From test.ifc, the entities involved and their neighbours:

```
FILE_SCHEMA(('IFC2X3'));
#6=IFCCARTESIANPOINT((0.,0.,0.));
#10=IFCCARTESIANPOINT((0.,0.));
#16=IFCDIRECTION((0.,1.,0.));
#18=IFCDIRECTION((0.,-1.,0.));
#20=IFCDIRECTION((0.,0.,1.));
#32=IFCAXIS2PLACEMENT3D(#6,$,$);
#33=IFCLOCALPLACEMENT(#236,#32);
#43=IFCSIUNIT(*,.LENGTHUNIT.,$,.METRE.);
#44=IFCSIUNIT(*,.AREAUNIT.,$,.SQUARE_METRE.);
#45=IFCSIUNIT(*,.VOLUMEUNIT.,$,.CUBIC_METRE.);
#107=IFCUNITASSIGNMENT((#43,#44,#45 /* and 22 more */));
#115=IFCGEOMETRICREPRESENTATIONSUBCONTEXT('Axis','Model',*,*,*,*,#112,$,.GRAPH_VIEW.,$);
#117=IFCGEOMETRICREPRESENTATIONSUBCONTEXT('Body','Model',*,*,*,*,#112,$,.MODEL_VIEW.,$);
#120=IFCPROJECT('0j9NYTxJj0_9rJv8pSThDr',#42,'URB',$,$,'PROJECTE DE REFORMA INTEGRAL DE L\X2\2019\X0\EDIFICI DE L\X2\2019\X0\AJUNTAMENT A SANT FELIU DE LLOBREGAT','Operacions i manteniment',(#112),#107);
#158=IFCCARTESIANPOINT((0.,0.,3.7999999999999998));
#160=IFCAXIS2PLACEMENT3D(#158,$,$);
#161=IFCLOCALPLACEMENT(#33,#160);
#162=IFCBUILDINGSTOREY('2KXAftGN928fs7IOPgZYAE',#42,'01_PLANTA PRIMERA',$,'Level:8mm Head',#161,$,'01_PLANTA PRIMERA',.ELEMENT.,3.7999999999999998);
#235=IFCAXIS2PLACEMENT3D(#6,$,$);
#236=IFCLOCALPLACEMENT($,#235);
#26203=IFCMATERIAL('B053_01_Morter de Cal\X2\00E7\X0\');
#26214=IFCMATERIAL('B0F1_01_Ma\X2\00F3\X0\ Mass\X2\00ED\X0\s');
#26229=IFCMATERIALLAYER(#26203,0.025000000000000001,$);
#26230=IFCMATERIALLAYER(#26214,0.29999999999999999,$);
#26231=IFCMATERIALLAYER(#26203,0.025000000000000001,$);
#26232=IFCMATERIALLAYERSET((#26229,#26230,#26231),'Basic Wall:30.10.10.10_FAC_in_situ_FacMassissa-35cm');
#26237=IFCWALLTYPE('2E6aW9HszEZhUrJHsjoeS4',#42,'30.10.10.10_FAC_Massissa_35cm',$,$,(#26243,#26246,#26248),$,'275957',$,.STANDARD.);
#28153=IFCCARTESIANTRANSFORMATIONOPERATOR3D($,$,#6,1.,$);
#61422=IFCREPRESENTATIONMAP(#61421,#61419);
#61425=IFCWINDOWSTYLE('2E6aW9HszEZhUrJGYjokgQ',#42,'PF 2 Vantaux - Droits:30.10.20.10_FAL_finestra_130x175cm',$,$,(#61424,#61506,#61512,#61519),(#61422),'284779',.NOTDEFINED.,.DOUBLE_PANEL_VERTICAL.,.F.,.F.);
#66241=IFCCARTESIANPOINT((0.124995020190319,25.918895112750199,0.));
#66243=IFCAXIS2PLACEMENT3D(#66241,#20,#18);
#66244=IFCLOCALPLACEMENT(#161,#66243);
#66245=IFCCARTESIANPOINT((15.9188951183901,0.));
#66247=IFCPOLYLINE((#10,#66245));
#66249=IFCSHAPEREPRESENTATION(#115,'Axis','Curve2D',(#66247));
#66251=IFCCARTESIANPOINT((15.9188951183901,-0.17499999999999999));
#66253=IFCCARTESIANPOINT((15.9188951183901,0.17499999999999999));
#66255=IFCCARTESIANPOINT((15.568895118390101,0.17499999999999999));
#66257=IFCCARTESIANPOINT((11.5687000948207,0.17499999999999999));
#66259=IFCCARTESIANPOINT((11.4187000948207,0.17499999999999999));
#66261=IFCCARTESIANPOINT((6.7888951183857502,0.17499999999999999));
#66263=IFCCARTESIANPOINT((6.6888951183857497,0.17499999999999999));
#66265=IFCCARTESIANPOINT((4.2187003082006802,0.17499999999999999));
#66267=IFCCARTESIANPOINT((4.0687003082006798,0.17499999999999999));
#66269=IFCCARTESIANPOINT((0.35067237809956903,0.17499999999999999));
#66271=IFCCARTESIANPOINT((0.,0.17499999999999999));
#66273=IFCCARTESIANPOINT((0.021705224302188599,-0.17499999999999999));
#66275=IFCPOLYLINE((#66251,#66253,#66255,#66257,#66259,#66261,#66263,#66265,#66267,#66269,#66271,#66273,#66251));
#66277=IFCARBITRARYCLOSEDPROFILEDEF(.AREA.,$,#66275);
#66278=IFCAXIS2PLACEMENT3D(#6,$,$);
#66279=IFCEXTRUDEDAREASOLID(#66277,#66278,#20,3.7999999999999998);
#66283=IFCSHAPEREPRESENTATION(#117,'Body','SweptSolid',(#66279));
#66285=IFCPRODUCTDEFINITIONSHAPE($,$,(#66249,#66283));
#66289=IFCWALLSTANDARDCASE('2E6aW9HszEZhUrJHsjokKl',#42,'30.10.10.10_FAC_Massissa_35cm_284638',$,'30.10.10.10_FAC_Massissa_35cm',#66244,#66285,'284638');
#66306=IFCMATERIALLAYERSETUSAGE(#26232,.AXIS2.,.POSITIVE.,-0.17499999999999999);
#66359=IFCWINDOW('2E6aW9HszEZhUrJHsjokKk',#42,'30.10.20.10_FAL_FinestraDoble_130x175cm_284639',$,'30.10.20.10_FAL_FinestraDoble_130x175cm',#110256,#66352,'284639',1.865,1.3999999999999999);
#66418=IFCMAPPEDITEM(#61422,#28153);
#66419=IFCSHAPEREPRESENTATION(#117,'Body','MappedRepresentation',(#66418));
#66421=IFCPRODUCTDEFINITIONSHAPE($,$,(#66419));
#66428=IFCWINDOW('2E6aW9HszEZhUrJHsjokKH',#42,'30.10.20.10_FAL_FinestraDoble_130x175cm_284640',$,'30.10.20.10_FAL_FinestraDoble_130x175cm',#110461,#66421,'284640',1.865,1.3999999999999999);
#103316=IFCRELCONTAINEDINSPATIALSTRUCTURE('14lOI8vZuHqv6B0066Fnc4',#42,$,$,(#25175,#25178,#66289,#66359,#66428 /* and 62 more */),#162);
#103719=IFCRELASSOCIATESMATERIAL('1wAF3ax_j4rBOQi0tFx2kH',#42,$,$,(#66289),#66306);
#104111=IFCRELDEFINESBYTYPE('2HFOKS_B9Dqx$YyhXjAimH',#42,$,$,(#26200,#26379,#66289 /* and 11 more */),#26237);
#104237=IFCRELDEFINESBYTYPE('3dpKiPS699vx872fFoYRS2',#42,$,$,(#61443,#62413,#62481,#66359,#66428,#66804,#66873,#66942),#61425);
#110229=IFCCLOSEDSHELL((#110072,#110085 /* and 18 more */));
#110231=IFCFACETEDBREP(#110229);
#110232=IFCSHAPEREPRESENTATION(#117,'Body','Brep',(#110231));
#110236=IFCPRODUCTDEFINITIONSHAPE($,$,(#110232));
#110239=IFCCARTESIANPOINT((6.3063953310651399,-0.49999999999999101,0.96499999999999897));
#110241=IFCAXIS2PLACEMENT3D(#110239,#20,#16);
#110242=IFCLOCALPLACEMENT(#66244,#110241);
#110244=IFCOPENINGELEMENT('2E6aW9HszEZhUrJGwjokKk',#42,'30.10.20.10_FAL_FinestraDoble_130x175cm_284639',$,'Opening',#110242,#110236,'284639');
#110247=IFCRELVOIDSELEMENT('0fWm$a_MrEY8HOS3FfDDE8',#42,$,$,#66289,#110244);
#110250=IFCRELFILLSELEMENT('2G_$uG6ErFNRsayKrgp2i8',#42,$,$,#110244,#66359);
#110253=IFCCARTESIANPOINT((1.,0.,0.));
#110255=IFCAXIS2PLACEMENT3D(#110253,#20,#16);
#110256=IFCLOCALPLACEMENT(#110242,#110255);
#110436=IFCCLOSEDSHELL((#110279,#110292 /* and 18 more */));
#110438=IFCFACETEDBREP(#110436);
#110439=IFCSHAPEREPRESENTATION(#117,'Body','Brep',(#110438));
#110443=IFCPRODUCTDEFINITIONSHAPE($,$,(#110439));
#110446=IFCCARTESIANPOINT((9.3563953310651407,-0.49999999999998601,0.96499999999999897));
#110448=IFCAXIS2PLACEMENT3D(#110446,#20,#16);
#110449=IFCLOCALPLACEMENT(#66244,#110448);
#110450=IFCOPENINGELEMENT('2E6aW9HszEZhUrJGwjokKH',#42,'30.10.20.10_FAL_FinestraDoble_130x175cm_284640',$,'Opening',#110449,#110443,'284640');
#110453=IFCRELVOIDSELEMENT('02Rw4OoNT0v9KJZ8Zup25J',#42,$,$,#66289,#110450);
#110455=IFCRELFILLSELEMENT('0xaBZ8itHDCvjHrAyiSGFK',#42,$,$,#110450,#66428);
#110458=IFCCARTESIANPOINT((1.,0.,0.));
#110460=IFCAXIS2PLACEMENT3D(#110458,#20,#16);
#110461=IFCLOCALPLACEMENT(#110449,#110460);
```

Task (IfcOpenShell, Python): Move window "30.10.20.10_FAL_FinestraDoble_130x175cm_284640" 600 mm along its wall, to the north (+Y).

```python
import ifcopenshell
import ifcopenshell.api.geometry
import ifcopenshell.util.placement
import ifcopenshell.util.unit

model = ifcopenshell.open("test.ifc")
unit_scale = ifcopenshell.util.unit.calculate_unit_scale(model)

window = model.by_guid("2E6aW9HszEZhUrJHsjokKH")
opening = window.FillsVoids[0].RelatingOpeningElement
wall = opening.VoidsElements[0].RelatingBuildingElement

wall_matrix = ifcopenshell.util.placement.get_local_placement(wall.ObjectPlacement)
shift = wall_matrix[:3, 0] * -0.6 / unit_scale
before = ifcopenshell.util.placement.get_local_placement(window.ObjectPlacement)[:3, 3].copy()

# The window is placed relative to its opening, so it follows when the opening moves.
matrix = ifcopenshell.util.placement.get_local_placement(opening.ObjectPlacement)
matrix[:3, 3] += shift
ifcopenshell.api.geometry.edit_object_placement(
    model, product=opening, matrix=matrix, is_si=False, should_transform_children=True
)

after = ifcopenshell.util.placement.get_local_placement(window.ObjectPlacement)[:3, 3]
print("window moved by", (after - before).round(3) + 0.0)

model.write("test_edited.ifc")
```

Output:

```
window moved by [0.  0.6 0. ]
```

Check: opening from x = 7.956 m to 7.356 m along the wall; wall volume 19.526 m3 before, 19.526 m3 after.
